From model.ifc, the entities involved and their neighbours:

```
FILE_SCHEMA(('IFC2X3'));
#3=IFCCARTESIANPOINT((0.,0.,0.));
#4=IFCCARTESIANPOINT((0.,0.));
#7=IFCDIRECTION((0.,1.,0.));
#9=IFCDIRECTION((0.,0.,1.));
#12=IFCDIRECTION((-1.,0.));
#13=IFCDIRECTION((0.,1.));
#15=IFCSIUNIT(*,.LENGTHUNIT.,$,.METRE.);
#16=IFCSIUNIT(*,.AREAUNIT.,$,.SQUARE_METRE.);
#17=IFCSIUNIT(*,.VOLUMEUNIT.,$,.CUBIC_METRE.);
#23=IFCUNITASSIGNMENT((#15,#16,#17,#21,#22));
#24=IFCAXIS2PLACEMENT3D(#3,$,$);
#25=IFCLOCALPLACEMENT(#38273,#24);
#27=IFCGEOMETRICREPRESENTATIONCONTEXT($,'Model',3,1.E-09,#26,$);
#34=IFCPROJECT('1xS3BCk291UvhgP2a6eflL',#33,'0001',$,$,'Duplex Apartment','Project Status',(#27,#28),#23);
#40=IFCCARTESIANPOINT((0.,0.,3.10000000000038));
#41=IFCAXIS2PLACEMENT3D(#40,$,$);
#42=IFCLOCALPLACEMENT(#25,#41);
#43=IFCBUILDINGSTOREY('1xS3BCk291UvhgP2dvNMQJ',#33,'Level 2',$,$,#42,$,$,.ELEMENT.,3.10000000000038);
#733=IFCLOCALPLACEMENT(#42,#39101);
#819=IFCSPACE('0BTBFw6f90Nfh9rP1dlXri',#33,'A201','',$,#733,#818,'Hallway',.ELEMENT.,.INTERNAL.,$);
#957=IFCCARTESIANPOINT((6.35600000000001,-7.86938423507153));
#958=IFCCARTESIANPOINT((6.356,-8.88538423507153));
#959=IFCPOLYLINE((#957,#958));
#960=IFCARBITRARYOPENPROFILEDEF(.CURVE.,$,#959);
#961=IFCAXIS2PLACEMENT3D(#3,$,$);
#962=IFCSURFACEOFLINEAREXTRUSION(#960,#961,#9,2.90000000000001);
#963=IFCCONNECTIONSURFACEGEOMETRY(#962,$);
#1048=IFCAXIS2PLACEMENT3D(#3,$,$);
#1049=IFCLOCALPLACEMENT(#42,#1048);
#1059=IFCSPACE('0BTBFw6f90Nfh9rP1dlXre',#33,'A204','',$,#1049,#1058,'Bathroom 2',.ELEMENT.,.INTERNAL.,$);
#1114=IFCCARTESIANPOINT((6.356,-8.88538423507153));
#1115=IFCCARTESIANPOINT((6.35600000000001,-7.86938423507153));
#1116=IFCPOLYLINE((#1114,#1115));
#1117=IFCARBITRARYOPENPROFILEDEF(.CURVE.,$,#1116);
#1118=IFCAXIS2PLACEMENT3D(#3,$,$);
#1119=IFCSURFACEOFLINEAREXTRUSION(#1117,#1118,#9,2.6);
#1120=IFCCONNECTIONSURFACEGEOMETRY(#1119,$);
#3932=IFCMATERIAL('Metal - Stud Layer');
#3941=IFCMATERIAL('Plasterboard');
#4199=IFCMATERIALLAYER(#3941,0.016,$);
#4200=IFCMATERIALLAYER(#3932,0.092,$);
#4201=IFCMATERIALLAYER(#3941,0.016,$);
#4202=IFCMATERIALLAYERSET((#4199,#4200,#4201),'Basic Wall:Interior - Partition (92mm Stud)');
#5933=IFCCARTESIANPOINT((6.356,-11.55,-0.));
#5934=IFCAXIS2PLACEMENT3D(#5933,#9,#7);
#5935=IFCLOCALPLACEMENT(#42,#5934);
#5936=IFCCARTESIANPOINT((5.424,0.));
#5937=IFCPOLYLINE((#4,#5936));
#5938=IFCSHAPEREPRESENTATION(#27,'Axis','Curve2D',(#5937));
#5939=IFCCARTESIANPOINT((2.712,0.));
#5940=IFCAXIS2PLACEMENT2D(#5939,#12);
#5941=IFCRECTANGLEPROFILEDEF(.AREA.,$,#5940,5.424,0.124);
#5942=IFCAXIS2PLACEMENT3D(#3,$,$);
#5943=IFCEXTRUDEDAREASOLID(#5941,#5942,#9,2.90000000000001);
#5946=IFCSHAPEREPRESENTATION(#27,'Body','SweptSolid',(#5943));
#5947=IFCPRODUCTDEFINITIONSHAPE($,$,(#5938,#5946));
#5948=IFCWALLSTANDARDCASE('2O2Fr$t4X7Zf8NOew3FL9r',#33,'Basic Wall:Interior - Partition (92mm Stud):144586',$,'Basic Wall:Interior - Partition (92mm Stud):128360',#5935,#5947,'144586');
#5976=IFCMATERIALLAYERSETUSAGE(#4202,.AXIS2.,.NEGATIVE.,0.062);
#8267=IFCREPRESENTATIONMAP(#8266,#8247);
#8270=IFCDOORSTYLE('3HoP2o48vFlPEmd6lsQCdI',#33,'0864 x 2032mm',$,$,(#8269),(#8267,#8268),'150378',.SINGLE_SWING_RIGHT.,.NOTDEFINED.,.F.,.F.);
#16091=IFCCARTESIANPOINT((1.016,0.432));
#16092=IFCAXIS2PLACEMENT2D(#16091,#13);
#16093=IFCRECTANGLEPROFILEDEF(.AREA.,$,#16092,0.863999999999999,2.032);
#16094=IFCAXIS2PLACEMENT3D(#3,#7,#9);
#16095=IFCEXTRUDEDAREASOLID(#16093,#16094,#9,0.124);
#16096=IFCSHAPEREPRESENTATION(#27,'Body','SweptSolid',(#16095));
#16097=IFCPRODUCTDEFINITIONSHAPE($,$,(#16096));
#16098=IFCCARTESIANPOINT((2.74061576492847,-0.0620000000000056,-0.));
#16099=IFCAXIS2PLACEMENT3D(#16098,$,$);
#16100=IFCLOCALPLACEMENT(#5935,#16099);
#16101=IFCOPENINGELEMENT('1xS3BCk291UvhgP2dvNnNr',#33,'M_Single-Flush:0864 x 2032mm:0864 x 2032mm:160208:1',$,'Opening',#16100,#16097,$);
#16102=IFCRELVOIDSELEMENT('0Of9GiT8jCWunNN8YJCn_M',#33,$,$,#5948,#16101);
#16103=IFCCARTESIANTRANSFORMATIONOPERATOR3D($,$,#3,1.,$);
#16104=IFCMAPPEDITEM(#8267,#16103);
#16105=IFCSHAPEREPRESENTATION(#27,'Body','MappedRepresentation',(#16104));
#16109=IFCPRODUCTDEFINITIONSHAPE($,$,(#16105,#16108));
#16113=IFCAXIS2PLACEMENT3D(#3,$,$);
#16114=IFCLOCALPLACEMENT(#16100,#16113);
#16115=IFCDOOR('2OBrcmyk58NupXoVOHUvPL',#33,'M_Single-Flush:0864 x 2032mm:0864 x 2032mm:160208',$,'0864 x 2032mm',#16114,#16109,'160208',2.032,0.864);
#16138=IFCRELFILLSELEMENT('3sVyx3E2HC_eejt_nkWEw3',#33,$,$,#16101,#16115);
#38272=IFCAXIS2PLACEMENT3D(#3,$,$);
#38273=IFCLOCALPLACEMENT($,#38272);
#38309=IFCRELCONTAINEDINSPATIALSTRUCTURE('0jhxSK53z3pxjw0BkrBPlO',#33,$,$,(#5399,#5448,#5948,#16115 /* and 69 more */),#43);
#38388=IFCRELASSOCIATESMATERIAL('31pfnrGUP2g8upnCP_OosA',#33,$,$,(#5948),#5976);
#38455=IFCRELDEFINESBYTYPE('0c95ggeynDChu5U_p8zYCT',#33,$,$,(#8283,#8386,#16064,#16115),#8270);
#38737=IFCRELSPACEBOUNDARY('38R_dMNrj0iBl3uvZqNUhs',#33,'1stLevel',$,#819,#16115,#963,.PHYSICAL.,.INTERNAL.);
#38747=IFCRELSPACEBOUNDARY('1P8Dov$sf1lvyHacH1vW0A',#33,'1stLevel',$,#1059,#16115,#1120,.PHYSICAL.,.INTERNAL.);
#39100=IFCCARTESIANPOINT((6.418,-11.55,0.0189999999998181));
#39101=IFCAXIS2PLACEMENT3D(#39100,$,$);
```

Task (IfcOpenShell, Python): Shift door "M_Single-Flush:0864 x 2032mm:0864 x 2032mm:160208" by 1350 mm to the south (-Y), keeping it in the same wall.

```python
import numpy as np
import ifcopenshell
import ifcopenshell.api.geometry
import ifcopenshell.util.placement

model = ifcopenshell.open("model.ifc")

door = model.by_guid("2OBrcmyk58NupXoVOHUvPL")
opening = door.FillsVoids[0].RelatingOpeningElement
wall = opening.VoidsElements[0].RelatingBuildingElement

wall_matrix = ifcopenshell.util.placement.get_local_placement(wall.ObjectPlacement)
shift = wall_matrix[:3, 0] * -1.35
before = ifcopenshell.util.placement.get_local_placement(door.ObjectPlacement)[:3, 3].copy()

# The door is placed relative to its opening, so it follows when the opening moves.
matrix = ifcopenshell.util.placement.get_local_placement(opening.ObjectPlacement)
matrix[:3, 3] += shift
ifcopenshell.api.geometry.edit_object_placement(
    model, product=opening, matrix=matrix, is_si=False, should_transform_children=True
)

# Space boundary surfaces are stored in each space's coordinates; move them too.
for rel in door.ProvidesBoundaries:
    if not rel.ConnectionGeometry:
        continue
    surface = rel.ConnectionGeometry.SurfaceOnRelatingElement
    space_matrix = ifcopenshell.util.placement.get_local_placement(rel.RelatingSpace.ObjectPlacement)
    point = np.array(surface.Position.Location.Coordinates) + space_matrix[:3, :3].T @ shift
    surface.Position = model.createIfcAxis2Placement3D(
        model.createIfcCartesianPoint(point.tolist()), surface.Position.Axis, surface.Position.RefDirection
    )

after = ifcopenshell.util.placement.get_local_placement(door.ObjectPlacement)[:3, 3]
print("door moved by", (after - before).round(3) + 0.0)

model.write("model_edited.ifc")
```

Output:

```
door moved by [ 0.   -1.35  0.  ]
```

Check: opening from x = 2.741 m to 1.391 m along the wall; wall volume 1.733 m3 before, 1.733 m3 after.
